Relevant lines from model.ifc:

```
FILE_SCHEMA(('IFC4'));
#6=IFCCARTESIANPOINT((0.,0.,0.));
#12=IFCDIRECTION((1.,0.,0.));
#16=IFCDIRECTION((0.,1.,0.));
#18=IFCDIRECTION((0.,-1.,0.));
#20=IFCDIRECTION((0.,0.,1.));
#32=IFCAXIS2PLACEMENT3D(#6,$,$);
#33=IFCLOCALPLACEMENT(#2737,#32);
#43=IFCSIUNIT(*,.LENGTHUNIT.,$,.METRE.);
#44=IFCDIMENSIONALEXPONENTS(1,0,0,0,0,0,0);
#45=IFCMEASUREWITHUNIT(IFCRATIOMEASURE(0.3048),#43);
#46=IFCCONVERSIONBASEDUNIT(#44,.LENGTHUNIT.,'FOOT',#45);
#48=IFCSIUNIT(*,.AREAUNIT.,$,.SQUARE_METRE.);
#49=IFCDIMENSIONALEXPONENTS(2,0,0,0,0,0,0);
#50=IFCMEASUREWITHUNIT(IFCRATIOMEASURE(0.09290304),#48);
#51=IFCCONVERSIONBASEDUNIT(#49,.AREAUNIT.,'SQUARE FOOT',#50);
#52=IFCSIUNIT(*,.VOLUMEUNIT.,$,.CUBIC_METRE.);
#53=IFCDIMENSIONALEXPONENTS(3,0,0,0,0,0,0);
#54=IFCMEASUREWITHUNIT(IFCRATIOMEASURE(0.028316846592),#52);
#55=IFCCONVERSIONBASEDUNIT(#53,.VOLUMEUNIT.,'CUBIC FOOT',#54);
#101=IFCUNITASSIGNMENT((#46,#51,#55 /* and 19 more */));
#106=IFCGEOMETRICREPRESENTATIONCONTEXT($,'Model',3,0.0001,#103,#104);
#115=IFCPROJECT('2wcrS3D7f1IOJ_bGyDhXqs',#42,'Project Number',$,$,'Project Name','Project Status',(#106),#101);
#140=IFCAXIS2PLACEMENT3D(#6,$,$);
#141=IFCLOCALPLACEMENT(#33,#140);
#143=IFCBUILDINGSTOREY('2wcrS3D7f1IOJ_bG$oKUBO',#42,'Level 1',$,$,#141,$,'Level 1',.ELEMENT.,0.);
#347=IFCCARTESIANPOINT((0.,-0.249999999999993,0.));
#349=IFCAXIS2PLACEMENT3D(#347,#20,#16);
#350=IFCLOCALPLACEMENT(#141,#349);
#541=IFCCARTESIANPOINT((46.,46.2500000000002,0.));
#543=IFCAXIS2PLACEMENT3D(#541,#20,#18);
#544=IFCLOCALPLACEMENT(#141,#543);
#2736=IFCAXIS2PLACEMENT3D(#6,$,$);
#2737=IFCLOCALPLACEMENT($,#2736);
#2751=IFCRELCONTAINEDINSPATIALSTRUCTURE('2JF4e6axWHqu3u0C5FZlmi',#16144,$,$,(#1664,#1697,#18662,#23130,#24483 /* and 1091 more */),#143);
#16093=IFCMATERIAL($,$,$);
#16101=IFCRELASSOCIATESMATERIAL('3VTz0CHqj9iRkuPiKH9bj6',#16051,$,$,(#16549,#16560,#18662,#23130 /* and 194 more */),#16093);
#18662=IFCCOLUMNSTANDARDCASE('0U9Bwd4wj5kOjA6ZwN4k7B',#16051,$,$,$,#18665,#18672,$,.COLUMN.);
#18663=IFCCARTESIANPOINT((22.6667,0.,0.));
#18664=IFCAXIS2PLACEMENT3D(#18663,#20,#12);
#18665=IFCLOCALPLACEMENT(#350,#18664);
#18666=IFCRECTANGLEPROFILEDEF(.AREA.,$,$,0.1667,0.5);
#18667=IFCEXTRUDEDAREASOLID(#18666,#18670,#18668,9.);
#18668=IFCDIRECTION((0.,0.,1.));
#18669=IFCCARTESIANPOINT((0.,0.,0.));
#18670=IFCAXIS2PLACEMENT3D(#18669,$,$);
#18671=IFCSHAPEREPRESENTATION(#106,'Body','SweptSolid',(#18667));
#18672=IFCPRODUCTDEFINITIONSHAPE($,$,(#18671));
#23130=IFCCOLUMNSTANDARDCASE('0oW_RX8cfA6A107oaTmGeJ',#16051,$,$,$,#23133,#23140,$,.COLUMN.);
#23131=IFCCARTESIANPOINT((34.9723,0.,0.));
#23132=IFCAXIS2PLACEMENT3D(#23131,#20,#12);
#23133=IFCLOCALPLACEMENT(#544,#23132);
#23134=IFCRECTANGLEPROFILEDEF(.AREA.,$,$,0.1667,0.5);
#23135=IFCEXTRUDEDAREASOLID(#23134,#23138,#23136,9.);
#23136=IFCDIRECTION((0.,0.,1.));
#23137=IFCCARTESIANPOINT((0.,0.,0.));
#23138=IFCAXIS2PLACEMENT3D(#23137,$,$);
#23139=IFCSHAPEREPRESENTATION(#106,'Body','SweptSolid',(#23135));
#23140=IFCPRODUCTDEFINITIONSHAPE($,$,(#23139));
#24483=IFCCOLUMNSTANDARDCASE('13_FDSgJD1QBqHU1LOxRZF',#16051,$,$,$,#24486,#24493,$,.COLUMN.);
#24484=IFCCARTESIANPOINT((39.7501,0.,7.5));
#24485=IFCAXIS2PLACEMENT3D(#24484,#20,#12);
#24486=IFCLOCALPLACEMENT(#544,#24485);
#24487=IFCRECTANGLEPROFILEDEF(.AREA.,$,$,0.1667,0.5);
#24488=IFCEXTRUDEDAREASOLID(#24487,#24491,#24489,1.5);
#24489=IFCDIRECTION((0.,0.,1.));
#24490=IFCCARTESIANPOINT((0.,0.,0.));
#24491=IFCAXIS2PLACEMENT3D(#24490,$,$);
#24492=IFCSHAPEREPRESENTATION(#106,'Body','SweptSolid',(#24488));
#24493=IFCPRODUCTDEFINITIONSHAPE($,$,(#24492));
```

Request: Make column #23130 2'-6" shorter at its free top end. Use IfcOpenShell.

```python
import ifcopenshell
import ifcopenshell.util.unit

model = ifcopenshell.open("model.ifc")
unit_scale = ifcopenshell.util.unit.calculate_unit_scale(model)

member = model.by_guid("0oW_RX8cfA6A107oaTmGeJ")
change = -30 * 0.0254 / unit_scale

# The extrusion runs towards the end named, so only its depth changes.
body = next(r for r in member.Representation.Representations if r.RepresentationIdentifier == "Body")
solid = body.Items[0]
old_length = solid.Depth
solid.Depth += change

print(f"length {old_length:g} -> {solid.Depth:g}")

model.write("model_updated.ifc")
```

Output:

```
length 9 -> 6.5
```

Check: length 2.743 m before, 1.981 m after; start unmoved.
